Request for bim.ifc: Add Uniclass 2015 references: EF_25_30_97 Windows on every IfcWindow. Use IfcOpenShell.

First a look at what the model holds.

```python
import ifcopenshell

model = ifcopenshell.open("bim.ifc")
print(model.schema)
print("classifications:", [c.Name for c in model.by_type("IfcClassification")])
for ifc_class in ("IfcDoor", "IfcRoof", "IfcStair", "IfcWall", "IfcWindow"):
    print(ifc_class, len(model.by_type(ifc_class)))
```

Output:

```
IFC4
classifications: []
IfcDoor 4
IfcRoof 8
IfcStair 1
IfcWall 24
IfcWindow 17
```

```python
import ifcopenshell
import ifcopenshell.api.classification

model = ifcopenshell.open("bim.ifc")

system = ifcopenshell.api.classification.add_classification(model, classification="Uniclass 2015")

codes = {
    "IfcWindow": ("EF_25_30_97", "Windows"),
}
for ifc_class, (code, name) in codes.items():
    products = model.by_type(ifc_class)
    ifcopenshell.api.classification.add_reference(
        model, products=products, classification=system, identification=code, name=name
    )
    print(code, len(products))

model.write("bim_updated.ifc")
```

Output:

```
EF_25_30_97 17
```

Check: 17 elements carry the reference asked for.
